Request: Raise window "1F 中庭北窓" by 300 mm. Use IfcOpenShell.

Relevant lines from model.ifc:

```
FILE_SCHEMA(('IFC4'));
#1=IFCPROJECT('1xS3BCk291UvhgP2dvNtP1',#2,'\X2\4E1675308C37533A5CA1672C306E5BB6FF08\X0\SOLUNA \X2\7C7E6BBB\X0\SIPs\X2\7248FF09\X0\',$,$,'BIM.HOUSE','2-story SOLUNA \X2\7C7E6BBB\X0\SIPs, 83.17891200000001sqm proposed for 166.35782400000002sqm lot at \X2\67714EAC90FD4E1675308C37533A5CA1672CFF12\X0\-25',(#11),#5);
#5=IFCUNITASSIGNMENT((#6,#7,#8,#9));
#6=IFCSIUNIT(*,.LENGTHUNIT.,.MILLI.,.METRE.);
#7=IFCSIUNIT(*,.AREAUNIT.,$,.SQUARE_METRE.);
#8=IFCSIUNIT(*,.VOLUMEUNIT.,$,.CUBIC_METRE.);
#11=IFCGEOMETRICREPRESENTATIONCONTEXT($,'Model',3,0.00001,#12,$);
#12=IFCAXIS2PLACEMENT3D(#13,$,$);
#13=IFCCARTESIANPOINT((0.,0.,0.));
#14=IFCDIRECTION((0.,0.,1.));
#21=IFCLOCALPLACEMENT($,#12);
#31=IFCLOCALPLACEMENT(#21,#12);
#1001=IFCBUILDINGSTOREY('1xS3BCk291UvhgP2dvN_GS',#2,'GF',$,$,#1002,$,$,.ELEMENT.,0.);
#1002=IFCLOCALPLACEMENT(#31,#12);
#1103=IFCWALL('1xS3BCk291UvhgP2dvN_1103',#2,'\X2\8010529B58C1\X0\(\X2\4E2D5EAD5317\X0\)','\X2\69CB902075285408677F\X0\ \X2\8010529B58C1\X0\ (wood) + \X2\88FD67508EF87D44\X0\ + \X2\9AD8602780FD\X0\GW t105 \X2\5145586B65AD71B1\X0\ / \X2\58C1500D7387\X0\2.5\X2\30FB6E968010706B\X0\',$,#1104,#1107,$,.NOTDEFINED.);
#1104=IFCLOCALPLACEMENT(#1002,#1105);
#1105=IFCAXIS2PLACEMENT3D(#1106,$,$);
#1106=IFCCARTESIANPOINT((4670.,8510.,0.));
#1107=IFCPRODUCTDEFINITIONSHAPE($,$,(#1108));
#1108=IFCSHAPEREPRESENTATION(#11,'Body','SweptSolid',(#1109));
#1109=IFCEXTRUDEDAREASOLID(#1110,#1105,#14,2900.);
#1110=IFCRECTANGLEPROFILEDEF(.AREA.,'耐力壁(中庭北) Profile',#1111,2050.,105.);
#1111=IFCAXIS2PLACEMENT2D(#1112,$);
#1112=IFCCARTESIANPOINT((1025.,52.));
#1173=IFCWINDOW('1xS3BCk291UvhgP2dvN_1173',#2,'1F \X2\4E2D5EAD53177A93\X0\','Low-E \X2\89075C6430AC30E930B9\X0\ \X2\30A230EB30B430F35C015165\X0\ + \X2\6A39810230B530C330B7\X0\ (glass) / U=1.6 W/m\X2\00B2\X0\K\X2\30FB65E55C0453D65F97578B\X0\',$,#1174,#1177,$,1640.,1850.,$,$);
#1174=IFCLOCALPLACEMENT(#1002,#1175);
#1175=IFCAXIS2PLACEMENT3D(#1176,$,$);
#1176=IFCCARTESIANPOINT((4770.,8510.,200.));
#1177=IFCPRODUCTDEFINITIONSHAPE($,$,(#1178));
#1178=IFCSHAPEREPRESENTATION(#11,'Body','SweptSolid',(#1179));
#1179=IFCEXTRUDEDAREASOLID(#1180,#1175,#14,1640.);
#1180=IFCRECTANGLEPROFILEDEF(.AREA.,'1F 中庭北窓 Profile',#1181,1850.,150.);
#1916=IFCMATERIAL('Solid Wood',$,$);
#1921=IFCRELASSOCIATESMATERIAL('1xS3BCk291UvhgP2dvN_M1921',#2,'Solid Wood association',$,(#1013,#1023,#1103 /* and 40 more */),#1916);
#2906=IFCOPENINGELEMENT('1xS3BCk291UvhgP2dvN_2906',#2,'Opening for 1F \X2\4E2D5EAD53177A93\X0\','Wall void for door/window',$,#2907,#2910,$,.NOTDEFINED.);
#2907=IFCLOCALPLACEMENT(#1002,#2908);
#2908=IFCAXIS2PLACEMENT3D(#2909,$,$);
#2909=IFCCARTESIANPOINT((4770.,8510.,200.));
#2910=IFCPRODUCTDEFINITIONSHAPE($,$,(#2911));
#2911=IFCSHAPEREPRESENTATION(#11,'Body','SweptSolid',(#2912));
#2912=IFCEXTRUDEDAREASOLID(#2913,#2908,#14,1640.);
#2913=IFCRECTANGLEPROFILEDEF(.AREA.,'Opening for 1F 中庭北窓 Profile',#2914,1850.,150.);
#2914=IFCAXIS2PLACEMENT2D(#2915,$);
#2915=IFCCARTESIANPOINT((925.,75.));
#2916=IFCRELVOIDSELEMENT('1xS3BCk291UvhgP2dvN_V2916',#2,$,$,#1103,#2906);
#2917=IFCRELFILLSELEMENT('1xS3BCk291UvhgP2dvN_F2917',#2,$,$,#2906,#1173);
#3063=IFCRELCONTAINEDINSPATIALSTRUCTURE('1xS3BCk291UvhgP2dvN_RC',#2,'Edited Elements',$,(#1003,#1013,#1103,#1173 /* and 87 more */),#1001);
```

```python
import numpy as np
import ifcopenshell
import ifcopenshell.api.geometry
import ifcopenshell.util.placement
import ifcopenshell.util.unit

model = ifcopenshell.open("model.ifc")
unit_scale = ifcopenshell.util.unit.calculate_unit_scale(model)

window = model.by_guid("1xS3BCk291UvhgP2dvN_1173")
opening = window.FillsVoids[0].RelatingOpeningElement
dz = 300.0

shift = np.array([0.0, 0.0, dz])
# The window is not placed relative to its opening, so move both.
for product in (opening, window):
    matrix = ifcopenshell.util.placement.get_local_placement(product.ObjectPlacement)
    matrix[:3, 3] += shift
    ifcopenshell.api.geometry.edit_object_placement(model, product=product, matrix=matrix, is_si=False)

print(f"moved by {dz * unit_scale:+.3f} m")

model.write("model_rev.ifc")
```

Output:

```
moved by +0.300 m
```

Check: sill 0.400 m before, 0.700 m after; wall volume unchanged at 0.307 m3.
